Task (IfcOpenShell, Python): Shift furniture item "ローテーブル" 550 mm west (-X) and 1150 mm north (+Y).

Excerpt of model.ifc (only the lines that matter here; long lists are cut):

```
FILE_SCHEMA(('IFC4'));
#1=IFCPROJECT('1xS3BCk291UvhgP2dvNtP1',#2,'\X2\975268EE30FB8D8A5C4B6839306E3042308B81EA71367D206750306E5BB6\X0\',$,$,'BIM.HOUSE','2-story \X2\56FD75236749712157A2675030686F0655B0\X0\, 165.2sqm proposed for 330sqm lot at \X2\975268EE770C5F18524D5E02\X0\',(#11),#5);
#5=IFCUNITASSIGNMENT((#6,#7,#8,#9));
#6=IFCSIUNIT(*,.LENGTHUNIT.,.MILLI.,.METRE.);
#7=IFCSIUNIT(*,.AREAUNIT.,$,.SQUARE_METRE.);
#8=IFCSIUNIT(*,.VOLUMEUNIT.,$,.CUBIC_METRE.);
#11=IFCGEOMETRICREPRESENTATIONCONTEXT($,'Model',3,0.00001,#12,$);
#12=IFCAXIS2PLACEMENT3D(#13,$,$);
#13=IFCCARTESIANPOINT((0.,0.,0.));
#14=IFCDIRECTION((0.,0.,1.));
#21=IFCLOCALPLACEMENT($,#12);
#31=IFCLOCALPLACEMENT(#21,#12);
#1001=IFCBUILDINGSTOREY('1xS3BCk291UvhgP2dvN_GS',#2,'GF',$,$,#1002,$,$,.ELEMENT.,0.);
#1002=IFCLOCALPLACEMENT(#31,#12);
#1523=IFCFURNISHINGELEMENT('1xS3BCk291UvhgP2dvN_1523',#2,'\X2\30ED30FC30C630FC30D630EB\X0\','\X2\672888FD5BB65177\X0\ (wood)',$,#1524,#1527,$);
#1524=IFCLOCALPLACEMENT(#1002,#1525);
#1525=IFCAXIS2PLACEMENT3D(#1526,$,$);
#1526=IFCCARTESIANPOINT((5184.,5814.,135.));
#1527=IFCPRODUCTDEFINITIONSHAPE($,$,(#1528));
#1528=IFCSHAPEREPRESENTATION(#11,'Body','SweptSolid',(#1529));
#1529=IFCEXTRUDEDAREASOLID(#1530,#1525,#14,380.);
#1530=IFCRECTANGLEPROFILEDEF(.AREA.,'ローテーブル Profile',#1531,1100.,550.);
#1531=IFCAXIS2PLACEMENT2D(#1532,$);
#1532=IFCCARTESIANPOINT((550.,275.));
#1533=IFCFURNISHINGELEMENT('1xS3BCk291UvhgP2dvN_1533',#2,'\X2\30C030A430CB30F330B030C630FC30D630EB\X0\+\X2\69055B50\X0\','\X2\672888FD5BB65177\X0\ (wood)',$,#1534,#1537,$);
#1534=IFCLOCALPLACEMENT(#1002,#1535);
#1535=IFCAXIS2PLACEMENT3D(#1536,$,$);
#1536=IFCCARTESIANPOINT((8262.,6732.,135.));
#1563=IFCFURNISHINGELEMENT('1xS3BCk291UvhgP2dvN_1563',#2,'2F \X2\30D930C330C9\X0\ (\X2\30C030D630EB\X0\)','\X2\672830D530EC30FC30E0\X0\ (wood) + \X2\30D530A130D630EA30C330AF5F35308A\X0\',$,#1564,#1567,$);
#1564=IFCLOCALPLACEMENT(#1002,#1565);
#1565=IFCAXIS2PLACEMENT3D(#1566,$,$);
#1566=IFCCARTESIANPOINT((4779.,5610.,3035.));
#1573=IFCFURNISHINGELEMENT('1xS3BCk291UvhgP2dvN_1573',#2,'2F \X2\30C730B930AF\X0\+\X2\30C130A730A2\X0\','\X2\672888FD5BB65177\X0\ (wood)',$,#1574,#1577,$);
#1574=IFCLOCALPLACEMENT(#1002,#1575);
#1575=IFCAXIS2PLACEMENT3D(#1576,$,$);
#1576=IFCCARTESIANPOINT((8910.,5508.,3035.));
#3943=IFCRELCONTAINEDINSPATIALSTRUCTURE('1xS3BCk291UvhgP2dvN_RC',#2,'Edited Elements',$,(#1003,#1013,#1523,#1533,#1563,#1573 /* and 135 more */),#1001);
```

```python
import ifcopenshell
import ifcopenshell.api.geometry
import ifcopenshell.util.placement
import ifcopenshell.util.unit

model = ifcopenshell.open("model.ifc")
unit_scale = ifcopenshell.util.unit.calculate_unit_scale(model)

item = model.by_id(1523)
matrix = ifcopenshell.util.placement.get_local_placement(item.ObjectPlacement)
matrix[0, 3] -= 0.55 / unit_scale
matrix[1, 3] += 1.15 / unit_scale
ifcopenshell.api.geometry.edit_object_placement(model, product=item, matrix=matrix, is_si=False)

print(ifcopenshell.util.placement.get_local_placement(item.ObjectPlacement).round(3) + 0.0)

model.write("model_rev.ifc")
```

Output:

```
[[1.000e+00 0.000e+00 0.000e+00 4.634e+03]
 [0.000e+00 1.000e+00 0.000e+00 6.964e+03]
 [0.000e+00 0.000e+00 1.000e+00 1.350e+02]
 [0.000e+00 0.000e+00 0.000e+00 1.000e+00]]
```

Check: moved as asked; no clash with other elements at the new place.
